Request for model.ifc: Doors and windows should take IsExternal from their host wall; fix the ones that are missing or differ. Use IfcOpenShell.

First a look at what the model holds.

```python
import ifcopenshell
import ifcopenshell.util.element

model = ifcopenshell.open("model.ifc")
print(model.schema)
seen = {}
for e in model.by_type("IfcDoor") + model.by_type("IfcWindow"):
    if not e.FillsVoids:
        continue
    host = e.FillsVoids[0].RelatingOpeningElement.VoidsElements[0].RelatingBuildingElement
    own = ifcopenshell.util.element.get_pset(e, f"Pset_{e.is_a()[3:].removesuffix('StandardCase')}Common", "IsExternal")
    wall = ifcopenshell.util.element.get_pset(host, "Pset_WallCommon", "IsExternal")
    seen[e.is_a(), own, wall] = seen.get((e.is_a(), own, wall), 0) + 1
for (cls, own, wall), count in sorted(seen.items(), key=str):
    print(count, cls, "IsExternal:", own, "| host wall:", wall)
```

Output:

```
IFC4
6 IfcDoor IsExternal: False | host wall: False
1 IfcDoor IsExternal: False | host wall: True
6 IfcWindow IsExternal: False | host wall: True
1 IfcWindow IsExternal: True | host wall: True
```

```python
import ifcopenshell
import ifcopenshell.api.pset
import ifcopenshell.util.element

model = ifcopenshell.open("model.ifc")

count = 0
for ifc_class, pset_name in (("IfcDoor", "Pset_DoorCommon"), ("IfcWindow", "Pset_WindowCommon")):
    for e in model.by_type(ifc_class):
        if not e.FillsVoids:
            continue
        host = e.FillsVoids[0].RelatingOpeningElement.VoidsElements[0].RelatingBuildingElement
        external = ifcopenshell.util.element.get_pset(host, "Pset_WallCommon", "IsExternal")
        if external is None or ifcopenshell.util.element.get_pset(e, pset_name, "IsExternal") == external:
            continue
        pset = ifcopenshell.api.pset.add_pset(model, product=e, name=pset_name)
        ifcopenshell.api.pset.edit_pset(model, pset=pset, properties={"IsExternal": external})
        count += 1

print(count, "updated")

model.write("model_updated.ifc")
```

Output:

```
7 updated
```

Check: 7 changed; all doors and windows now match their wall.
